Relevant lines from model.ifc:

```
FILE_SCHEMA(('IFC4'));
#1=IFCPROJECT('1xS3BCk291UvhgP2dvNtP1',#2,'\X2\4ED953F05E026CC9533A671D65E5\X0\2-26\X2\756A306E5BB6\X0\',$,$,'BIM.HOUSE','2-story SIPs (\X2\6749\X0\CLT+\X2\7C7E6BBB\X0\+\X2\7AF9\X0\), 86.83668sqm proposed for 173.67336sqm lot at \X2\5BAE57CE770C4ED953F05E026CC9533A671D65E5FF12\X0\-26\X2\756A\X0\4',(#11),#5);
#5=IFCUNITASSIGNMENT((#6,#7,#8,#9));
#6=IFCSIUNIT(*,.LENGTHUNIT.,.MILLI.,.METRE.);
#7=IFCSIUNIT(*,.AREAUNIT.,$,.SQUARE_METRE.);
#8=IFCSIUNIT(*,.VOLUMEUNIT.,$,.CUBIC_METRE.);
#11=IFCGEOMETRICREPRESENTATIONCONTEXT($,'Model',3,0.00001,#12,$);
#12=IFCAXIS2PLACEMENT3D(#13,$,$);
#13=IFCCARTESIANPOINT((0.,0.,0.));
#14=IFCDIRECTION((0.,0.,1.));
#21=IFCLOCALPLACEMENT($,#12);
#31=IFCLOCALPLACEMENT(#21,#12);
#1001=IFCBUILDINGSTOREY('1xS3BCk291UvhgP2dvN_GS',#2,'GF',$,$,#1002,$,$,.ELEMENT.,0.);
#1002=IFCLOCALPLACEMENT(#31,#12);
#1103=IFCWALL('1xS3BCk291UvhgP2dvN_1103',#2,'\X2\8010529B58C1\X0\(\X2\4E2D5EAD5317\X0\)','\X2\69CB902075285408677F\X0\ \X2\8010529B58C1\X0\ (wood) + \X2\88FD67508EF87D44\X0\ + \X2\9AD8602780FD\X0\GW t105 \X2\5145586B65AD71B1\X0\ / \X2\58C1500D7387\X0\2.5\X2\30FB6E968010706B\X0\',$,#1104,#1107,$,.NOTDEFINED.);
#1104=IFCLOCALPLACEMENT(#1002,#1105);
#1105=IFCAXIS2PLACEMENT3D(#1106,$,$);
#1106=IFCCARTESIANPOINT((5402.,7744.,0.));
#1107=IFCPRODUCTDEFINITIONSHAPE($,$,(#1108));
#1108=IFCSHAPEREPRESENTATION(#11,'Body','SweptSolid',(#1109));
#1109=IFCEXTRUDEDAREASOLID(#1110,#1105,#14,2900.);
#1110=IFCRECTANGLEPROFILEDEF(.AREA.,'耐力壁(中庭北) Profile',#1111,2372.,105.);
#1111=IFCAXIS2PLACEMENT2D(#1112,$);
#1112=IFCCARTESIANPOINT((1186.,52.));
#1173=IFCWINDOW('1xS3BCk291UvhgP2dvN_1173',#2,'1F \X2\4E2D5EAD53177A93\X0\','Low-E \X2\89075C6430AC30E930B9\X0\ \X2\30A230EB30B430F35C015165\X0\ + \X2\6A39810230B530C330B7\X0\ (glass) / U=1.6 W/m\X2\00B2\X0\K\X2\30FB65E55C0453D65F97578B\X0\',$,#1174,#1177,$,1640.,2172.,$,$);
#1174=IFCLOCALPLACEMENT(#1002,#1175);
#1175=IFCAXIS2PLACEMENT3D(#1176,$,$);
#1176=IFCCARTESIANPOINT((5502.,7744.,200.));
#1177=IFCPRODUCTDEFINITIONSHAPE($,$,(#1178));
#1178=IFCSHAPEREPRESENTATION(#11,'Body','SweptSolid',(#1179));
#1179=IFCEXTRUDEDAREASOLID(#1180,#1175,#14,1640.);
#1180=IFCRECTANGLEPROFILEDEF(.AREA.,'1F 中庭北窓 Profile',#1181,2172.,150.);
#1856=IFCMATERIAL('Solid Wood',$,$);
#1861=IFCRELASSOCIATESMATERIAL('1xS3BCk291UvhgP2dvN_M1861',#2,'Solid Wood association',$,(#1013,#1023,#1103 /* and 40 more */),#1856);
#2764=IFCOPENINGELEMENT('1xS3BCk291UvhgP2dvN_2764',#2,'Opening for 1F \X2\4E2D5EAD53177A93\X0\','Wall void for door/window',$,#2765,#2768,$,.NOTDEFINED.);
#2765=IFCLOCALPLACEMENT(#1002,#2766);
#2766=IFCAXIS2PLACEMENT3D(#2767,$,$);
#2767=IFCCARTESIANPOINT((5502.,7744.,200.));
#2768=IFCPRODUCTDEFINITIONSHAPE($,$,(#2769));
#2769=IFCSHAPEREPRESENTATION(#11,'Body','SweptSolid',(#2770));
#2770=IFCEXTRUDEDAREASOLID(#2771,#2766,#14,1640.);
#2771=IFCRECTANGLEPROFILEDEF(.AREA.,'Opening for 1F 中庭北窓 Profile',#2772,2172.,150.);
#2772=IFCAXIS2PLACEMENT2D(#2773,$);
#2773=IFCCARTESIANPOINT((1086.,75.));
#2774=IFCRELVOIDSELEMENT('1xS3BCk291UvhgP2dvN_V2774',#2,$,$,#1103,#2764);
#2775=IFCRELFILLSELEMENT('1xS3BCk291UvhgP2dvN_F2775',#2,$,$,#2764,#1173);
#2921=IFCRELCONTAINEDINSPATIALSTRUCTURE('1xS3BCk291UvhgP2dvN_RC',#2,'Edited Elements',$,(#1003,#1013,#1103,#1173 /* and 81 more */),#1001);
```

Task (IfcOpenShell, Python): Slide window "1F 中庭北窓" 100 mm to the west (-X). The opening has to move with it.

```python
import ifcopenshell
import ifcopenshell.api.geometry
import ifcopenshell.util.placement
import ifcopenshell.util.unit

model = ifcopenshell.open("model.ifc")
unit_scale = ifcopenshell.util.unit.calculate_unit_scale(model)

window = model.by_id(1173)
opening = window.FillsVoids[0].RelatingOpeningElement
wall = opening.VoidsElements[0].RelatingBuildingElement

wall_matrix = ifcopenshell.util.placement.get_local_placement(wall.ObjectPlacement)
shift = wall_matrix[:3, 0] * -0.1 / unit_scale
before = ifcopenshell.util.placement.get_local_placement(window.ObjectPlacement)[:3, 3].copy()

# The window is not placed relative to its opening, so move both.
for product in (opening, window):
    matrix = ifcopenshell.util.placement.get_local_placement(product.ObjectPlacement)
    matrix[:3, 3] += shift
    ifcopenshell.api.geometry.edit_object_placement(model, product=product, matrix=matrix, is_si=False)

after = ifcopenshell.util.placement.get_local_placement(window.ObjectPlacement)[:3, 3]
print("window moved by", (after - before).round(3) + 0.0)

model.write("model_edited.ifc")
```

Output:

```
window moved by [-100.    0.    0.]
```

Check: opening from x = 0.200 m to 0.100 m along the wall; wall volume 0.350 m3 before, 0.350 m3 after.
